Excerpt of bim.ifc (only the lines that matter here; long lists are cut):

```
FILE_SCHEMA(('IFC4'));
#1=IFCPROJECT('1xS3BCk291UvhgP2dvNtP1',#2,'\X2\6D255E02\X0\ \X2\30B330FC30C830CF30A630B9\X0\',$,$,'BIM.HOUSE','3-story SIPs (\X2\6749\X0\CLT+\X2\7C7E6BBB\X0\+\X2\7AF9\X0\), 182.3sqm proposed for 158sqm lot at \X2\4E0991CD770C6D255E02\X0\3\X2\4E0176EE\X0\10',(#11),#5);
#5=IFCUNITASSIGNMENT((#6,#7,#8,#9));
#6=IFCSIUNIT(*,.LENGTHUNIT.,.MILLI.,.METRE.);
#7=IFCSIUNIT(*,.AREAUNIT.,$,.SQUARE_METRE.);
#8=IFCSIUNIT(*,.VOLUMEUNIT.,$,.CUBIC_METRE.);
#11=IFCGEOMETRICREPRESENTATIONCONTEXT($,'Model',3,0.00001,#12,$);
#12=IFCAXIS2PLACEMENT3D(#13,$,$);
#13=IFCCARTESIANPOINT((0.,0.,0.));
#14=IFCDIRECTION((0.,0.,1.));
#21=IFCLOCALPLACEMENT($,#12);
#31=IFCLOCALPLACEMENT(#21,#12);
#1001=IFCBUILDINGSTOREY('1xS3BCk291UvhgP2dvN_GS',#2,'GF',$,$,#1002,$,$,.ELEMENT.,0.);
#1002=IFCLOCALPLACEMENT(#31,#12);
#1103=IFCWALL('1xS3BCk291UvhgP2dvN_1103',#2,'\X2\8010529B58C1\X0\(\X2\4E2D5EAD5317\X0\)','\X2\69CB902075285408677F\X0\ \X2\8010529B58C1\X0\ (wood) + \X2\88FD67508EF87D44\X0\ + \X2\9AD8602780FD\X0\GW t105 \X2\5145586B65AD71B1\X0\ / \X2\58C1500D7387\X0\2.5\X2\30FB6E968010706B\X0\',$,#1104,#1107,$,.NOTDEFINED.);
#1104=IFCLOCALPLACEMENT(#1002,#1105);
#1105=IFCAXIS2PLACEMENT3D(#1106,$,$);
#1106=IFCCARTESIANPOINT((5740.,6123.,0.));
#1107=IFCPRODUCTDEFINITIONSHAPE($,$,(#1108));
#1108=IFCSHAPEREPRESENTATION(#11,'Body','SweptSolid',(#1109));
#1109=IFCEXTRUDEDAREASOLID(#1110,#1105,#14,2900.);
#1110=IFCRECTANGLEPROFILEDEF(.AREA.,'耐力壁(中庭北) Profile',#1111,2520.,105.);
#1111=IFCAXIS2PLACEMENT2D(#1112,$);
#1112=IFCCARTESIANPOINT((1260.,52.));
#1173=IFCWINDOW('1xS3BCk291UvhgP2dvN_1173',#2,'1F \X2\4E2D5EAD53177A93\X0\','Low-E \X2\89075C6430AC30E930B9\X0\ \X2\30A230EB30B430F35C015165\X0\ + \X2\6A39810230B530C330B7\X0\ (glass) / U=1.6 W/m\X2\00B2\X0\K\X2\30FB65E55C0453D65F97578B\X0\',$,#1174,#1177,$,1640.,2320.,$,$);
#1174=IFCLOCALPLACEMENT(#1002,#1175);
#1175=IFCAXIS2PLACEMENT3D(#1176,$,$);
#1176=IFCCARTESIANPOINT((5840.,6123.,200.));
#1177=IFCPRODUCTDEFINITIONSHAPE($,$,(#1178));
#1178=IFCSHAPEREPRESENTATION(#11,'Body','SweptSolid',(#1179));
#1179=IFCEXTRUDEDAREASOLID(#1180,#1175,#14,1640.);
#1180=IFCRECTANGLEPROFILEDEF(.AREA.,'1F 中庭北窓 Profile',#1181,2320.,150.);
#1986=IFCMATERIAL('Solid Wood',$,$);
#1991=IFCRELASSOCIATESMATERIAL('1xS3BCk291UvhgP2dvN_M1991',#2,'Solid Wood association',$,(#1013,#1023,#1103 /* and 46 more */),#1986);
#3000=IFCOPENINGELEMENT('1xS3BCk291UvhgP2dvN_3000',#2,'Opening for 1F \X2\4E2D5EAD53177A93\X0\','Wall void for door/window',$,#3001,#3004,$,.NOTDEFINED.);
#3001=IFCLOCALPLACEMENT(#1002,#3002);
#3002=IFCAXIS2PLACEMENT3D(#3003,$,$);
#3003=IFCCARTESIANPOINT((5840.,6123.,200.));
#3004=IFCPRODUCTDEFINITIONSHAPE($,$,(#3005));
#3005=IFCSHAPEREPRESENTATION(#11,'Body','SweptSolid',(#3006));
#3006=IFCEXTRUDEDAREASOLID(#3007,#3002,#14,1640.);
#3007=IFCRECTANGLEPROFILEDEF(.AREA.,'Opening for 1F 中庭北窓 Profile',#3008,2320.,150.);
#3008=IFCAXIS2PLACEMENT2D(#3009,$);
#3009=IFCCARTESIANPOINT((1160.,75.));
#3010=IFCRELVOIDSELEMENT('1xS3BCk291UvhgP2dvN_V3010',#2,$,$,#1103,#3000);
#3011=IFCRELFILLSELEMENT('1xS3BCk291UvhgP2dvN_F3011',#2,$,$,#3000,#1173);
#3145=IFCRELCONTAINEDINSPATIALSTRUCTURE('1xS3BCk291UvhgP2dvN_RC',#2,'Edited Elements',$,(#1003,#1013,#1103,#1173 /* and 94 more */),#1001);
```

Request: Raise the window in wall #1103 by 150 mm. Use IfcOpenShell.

```python
import numpy as np
import ifcopenshell
import ifcopenshell.api.geometry
import ifcopenshell.util.placement
import ifcopenshell.util.unit

model = ifcopenshell.open("bim.ifc")
unit_scale = ifcopenshell.util.unit.calculate_unit_scale(model)

window = model.by_guid("1xS3BCk291UvhgP2dvN_1173")
opening = window.FillsVoids[0].RelatingOpeningElement
dz = 0.15 / unit_scale

shift = np.array([0.0, 0.0, dz])
# The window is not placed relative to its opening, so move both.
for product in (opening, window):
    matrix = ifcopenshell.util.placement.get_local_placement(product.ObjectPlacement)
    matrix[:3, 3] += shift
    ifcopenshell.api.geometry.edit_object_placement(model, product=product, matrix=matrix, is_si=False)

print(f"moved by {dz * unit_scale:+.3f} m")

model.write("bim_edited.ifc")
```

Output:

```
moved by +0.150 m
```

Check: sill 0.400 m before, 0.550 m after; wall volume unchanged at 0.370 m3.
